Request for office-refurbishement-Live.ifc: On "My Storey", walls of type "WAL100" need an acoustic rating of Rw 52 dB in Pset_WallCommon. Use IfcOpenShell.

First a look at what the model holds.

```python
import ifcopenshell
import ifcopenshell.util.element

model = ifcopenshell.open("office-refurbishement-Live.ifc")
print(model.schema)
storey = next(s for s in model.by_type("IfcBuildingStorey") if s.Name == "My Storey")
walls = [e for e in ifcopenshell.util.element.get_decomposition(storey) if e.is_a("IfcWall")]
seen = {}
for e in walls:
    element_type = ifcopenshell.util.element.get_type(e)
    key = (element_type.Name if element_type != e and element_type else None, ifcopenshell.util.element.get_pset(e, "Pset_WallCommon", "AcousticRating"))
    seen[key] = seen.get(key, 0) + 1
for (name, value), count in sorted(seen.items(), key=str):
    print(count, "x", name, "|", value)
```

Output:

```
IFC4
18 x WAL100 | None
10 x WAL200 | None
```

```python
import ifcopenshell
import ifcopenshell.api.pset
import ifcopenshell.util.element

model = ifcopenshell.open("office-refurbishement-Live.ifc")

storey = next(s for s in model.by_type("IfcBuildingStorey") if s.Name == "My Storey")
walls = [e for e in ifcopenshell.util.element.get_decomposition(storey) if e.is_a("IfcWall")]

count = 0
for e in walls:
    element_type = ifcopenshell.util.element.get_type(e)
    if element_type in (None, e) or element_type.Name != "WAL100":
        continue
    # add_pset returns the element's existing set when there is one.
    pset = ifcopenshell.api.pset.add_pset(model, product=e, name="Pset_WallCommon")
    ifcopenshell.api.pset.edit_pset(model, pset=pset, properties={"AcousticRating": "Rw 52 dB"})
    count += 1

print(count, "walls updated")

model.write("office-refurbishement-Live-out.ifc")
```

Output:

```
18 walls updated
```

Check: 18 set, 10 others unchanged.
